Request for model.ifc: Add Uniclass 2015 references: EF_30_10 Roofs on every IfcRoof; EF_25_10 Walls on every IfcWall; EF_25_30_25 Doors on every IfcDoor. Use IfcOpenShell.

First a look at what the model holds.

```python
import ifcopenshell

model = ifcopenshell.open("model.ifc")
print(model.schema)
print("classifications:", [c.Name for c in model.by_type("IfcClassification")])
for ifc_class in ("IfcDoor", "IfcRoof", "IfcStair", "IfcWall", "IfcWindow"):
    print(ifc_class, len(model.by_type(ifc_class)))
```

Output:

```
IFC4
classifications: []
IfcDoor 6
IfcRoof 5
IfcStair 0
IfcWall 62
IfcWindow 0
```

```python
import ifcopenshell
import ifcopenshell.api.classification

model = ifcopenshell.open("model.ifc")

system = ifcopenshell.api.classification.add_classification(model, classification="Uniclass 2015")

codes = {
    "IfcRoof": ("EF_30_10", "Roofs"),
    "IfcWall": ("EF_25_10", "Walls"),
    "IfcDoor": ("EF_25_30_25", "Doors"),
}
for ifc_class, (code, name) in codes.items():
    products = model.by_type(ifc_class)
    ifcopenshell.api.classification.add_reference(
        model, products=products, classification=system, identification=code, name=name
    )
    print(code, len(products))

model.write("model_v2.ifc")
```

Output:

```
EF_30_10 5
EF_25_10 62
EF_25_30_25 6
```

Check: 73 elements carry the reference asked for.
